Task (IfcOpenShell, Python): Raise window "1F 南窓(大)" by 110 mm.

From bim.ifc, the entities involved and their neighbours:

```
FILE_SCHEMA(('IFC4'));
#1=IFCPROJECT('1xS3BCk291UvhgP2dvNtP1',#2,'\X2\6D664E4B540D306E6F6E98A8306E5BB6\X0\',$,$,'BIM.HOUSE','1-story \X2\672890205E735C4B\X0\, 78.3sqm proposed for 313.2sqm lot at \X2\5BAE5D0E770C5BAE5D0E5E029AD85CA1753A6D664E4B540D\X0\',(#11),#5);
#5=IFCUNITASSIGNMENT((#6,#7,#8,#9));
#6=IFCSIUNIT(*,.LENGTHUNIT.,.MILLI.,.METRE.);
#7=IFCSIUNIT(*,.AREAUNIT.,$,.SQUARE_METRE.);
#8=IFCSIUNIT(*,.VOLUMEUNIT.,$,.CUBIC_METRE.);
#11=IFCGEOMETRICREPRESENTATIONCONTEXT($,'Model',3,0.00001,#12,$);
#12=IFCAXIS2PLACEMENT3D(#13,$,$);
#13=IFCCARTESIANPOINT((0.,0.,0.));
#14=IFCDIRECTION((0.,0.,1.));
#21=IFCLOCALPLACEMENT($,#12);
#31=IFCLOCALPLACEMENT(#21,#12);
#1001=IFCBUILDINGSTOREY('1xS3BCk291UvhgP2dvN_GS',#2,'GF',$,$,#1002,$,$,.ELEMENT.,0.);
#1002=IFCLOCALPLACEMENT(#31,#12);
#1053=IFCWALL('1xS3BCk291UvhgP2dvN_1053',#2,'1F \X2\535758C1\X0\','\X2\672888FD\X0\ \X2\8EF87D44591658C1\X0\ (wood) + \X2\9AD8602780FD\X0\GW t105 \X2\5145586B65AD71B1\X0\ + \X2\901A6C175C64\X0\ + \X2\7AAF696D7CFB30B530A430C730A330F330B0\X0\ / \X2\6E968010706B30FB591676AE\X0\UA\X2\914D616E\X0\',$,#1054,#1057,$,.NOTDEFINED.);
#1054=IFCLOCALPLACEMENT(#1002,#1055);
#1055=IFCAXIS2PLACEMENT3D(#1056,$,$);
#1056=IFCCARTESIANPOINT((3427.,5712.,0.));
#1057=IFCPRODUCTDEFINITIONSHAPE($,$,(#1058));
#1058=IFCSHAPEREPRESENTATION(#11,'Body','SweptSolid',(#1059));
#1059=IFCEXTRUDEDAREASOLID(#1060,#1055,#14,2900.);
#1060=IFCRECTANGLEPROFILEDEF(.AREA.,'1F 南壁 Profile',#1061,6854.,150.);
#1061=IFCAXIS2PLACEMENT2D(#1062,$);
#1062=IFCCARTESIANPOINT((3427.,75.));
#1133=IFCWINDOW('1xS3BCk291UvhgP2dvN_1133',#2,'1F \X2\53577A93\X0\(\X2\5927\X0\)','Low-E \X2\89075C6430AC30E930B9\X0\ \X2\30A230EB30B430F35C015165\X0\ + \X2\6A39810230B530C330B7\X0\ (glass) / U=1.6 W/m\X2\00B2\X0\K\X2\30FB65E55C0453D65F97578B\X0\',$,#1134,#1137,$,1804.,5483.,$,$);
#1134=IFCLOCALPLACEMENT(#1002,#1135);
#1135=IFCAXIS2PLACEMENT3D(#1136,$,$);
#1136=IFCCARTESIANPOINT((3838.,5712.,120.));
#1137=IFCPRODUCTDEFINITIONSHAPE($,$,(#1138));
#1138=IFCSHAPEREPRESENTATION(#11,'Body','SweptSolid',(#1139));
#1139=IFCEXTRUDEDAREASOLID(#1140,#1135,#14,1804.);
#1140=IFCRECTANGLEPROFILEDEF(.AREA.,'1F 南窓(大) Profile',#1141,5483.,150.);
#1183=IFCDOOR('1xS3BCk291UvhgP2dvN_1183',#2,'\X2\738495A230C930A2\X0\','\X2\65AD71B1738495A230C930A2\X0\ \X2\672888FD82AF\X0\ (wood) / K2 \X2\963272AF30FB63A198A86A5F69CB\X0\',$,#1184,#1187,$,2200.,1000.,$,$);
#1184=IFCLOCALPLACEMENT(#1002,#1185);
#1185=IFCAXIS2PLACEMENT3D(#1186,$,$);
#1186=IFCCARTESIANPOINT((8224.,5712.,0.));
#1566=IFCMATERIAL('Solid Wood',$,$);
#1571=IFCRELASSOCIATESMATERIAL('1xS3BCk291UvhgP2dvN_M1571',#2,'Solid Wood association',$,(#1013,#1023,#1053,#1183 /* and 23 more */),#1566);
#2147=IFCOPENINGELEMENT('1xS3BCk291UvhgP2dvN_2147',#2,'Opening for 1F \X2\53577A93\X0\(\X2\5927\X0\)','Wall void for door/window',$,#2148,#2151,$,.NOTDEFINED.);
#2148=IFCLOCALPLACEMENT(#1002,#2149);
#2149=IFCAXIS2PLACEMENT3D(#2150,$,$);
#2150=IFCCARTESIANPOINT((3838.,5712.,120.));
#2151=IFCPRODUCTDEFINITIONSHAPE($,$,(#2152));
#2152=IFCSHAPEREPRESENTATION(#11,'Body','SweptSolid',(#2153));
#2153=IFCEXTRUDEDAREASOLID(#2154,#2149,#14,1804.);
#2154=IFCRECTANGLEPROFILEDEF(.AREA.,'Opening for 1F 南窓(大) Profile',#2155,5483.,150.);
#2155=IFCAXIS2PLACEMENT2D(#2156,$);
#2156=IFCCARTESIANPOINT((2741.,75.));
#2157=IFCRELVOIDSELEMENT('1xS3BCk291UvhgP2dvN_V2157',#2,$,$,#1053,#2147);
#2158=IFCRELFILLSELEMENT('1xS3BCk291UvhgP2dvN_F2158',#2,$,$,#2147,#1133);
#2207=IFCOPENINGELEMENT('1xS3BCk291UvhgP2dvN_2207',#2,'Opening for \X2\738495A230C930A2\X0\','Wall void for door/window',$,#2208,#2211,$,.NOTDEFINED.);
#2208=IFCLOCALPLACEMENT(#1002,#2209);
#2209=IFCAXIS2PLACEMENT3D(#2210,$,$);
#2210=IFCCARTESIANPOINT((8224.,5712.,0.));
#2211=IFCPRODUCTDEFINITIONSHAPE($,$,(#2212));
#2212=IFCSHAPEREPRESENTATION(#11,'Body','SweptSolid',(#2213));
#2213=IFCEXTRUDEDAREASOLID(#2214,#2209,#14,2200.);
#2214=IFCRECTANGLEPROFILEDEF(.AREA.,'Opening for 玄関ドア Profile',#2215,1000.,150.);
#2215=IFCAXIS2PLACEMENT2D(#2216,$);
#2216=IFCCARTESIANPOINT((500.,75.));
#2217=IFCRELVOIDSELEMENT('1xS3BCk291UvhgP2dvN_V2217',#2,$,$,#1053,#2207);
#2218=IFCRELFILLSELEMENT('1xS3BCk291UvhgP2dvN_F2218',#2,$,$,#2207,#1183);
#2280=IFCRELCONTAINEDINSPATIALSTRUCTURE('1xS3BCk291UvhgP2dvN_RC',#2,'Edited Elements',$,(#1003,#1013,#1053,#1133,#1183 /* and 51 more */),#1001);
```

```python
import numpy as np
import ifcopenshell
import ifcopenshell.api.geometry
import ifcopenshell.util.placement
import ifcopenshell.util.unit

model = ifcopenshell.open("bim.ifc")
unit_scale = ifcopenshell.util.unit.calculate_unit_scale(model)

window = model.by_guid("1xS3BCk291UvhgP2dvN_1133")
opening = window.FillsVoids[0].RelatingOpeningElement
dz = 110.0

shift = np.array([0.0, 0.0, dz])
# The window is not placed relative to its opening, so move both.
for product in (opening, window):
    matrix = ifcopenshell.util.placement.get_local_placement(product.ObjectPlacement)
    matrix[:3, 3] += shift
    ifcopenshell.api.geometry.edit_object_placement(model, product=product, matrix=matrix, is_si=False)

print(f"moved by {dz * unit_scale:+.3f} m")

model.write("bim_rev.ifc")
```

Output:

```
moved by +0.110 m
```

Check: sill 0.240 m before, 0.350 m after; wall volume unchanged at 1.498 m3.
